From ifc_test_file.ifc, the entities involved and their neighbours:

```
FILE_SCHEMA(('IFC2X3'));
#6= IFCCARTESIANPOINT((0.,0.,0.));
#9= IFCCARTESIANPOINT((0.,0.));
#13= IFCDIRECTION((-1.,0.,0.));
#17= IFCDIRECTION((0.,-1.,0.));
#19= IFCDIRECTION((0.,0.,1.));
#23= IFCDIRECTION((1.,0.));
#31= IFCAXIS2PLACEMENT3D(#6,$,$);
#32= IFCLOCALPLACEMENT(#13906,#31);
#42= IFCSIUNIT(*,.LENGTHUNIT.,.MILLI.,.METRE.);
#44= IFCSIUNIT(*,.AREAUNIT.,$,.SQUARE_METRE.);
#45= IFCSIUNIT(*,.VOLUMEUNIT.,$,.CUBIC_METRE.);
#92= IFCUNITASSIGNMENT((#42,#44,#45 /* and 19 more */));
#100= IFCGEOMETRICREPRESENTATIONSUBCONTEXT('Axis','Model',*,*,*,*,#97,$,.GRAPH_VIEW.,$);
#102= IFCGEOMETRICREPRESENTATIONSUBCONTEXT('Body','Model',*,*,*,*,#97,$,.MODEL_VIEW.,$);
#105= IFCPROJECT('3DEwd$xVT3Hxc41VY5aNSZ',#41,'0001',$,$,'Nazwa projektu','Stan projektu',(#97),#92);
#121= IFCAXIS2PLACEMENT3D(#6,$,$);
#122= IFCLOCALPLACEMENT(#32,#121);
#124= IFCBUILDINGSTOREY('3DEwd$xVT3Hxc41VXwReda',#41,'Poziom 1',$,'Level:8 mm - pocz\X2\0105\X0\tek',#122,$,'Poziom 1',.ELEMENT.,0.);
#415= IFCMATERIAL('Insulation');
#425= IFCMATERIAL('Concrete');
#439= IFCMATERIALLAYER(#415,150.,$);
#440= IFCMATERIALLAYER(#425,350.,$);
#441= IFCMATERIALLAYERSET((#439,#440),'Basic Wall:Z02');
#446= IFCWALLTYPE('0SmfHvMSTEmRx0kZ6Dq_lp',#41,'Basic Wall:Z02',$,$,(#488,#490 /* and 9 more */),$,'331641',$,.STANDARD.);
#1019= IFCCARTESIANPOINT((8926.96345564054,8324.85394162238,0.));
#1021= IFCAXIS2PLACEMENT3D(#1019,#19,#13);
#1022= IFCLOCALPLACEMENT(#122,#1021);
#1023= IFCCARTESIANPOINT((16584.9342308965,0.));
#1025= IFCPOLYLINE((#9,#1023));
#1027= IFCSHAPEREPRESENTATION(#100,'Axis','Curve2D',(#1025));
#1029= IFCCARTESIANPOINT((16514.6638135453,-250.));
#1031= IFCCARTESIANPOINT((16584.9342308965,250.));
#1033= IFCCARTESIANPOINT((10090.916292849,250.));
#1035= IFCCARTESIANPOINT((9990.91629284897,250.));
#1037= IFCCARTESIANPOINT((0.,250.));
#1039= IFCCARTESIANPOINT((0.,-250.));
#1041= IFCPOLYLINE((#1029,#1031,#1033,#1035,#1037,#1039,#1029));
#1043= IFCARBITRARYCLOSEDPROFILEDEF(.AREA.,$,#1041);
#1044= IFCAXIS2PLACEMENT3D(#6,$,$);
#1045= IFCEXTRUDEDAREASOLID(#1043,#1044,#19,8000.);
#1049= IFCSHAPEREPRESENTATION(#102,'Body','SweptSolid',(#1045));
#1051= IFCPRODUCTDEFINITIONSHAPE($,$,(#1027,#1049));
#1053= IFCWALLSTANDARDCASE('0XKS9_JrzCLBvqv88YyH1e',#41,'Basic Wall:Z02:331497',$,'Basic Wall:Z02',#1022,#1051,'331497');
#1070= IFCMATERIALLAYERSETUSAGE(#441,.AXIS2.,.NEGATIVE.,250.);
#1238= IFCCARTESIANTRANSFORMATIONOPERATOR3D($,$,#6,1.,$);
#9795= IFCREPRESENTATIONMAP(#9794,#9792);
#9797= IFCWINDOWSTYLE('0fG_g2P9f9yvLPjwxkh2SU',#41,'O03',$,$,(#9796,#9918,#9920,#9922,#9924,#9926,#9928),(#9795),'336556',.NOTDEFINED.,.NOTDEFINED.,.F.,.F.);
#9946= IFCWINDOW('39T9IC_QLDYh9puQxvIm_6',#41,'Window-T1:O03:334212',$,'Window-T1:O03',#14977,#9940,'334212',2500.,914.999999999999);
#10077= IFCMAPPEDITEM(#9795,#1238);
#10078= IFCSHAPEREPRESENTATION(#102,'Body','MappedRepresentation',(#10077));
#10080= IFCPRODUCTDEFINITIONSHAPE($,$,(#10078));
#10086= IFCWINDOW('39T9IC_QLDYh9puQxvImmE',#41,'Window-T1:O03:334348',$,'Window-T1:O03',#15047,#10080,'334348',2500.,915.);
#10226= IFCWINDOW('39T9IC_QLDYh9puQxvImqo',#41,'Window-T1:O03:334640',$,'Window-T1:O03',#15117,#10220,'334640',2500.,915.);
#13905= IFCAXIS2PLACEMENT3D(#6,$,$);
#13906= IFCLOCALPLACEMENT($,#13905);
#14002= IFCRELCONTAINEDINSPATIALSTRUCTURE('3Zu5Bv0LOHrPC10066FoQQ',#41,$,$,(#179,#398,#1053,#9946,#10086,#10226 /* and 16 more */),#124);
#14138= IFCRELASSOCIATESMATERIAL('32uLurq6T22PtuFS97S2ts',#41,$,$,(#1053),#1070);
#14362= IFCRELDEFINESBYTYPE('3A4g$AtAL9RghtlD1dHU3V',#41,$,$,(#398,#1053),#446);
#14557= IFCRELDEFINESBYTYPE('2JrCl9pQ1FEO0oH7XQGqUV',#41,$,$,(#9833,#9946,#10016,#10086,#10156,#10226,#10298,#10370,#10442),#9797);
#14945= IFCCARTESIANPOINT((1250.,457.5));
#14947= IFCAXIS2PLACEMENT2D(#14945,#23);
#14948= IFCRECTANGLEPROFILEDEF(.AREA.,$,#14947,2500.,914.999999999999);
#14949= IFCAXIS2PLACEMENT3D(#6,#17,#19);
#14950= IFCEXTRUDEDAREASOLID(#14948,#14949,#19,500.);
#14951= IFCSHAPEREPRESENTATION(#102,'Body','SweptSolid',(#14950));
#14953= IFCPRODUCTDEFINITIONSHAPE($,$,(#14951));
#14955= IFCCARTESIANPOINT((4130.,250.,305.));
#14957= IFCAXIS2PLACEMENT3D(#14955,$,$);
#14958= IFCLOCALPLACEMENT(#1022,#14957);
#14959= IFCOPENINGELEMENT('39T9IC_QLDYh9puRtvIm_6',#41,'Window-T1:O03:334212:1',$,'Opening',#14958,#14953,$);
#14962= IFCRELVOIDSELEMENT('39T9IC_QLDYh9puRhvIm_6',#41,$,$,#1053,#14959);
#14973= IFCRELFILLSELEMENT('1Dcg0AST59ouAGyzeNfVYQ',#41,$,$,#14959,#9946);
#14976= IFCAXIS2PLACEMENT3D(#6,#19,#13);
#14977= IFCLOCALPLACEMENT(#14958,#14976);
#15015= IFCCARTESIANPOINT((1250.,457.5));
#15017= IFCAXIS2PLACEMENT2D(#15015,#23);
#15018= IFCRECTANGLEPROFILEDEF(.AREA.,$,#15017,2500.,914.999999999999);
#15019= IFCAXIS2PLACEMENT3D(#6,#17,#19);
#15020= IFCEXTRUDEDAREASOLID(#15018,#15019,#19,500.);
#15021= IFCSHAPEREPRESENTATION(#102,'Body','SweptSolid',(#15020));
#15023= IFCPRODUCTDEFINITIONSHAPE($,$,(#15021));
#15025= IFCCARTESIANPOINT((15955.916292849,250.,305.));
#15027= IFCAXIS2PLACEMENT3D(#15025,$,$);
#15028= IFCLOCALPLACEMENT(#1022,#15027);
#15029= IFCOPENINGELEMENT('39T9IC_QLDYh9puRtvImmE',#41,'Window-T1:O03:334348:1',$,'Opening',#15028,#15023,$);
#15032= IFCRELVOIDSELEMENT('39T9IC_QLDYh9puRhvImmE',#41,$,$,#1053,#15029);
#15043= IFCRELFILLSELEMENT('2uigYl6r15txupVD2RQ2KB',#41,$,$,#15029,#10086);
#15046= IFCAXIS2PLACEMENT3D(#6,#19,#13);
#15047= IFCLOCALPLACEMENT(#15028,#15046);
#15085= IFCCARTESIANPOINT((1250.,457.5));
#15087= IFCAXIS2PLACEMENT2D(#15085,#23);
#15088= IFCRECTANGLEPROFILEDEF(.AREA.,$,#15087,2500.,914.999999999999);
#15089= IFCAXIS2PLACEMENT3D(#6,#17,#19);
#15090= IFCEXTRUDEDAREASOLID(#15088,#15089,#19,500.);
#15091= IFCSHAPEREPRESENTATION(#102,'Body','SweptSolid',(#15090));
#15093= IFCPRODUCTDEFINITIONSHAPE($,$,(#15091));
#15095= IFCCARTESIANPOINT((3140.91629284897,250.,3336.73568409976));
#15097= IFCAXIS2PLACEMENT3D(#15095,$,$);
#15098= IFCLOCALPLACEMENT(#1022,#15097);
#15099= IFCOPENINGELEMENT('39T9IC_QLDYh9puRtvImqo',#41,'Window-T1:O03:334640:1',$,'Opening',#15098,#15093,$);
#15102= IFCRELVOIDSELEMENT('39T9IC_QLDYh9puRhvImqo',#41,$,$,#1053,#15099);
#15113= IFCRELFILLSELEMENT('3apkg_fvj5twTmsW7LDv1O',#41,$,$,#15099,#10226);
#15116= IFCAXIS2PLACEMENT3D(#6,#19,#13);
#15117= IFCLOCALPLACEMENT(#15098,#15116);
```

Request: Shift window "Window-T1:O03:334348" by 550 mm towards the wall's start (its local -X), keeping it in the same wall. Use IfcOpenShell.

```python
import ifcopenshell
import ifcopenshell.api.geometry
import ifcopenshell.util.placement

model = ifcopenshell.open("ifc_test_file.ifc")

window = model.by_id(10086)
opening = window.FillsVoids[0].RelatingOpeningElement
wall = opening.VoidsElements[0].RelatingBuildingElement

wall_matrix = ifcopenshell.util.placement.get_local_placement(wall.ObjectPlacement)
shift = wall_matrix[:3, 0] * -550.0
before = ifcopenshell.util.placement.get_local_placement(window.ObjectPlacement)[:3, 3].copy()

# The window is placed relative to its opening, so it follows when the opening moves.
matrix = ifcopenshell.util.placement.get_local_placement(opening.ObjectPlacement)
matrix[:3, 3] += shift
ifcopenshell.api.geometry.edit_object_placement(
    model, product=opening, matrix=matrix, is_si=False, should_transform_children=True
)

after = ifcopenshell.util.placement.get_local_placement(window.ObjectPlacement)[:3, 3]
print("window moved by", (after - before).round(3) + 0.0)

model.write("ifc_test_file_edited.ifc")
```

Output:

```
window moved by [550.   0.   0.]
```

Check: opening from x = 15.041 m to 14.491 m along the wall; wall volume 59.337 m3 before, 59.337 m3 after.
